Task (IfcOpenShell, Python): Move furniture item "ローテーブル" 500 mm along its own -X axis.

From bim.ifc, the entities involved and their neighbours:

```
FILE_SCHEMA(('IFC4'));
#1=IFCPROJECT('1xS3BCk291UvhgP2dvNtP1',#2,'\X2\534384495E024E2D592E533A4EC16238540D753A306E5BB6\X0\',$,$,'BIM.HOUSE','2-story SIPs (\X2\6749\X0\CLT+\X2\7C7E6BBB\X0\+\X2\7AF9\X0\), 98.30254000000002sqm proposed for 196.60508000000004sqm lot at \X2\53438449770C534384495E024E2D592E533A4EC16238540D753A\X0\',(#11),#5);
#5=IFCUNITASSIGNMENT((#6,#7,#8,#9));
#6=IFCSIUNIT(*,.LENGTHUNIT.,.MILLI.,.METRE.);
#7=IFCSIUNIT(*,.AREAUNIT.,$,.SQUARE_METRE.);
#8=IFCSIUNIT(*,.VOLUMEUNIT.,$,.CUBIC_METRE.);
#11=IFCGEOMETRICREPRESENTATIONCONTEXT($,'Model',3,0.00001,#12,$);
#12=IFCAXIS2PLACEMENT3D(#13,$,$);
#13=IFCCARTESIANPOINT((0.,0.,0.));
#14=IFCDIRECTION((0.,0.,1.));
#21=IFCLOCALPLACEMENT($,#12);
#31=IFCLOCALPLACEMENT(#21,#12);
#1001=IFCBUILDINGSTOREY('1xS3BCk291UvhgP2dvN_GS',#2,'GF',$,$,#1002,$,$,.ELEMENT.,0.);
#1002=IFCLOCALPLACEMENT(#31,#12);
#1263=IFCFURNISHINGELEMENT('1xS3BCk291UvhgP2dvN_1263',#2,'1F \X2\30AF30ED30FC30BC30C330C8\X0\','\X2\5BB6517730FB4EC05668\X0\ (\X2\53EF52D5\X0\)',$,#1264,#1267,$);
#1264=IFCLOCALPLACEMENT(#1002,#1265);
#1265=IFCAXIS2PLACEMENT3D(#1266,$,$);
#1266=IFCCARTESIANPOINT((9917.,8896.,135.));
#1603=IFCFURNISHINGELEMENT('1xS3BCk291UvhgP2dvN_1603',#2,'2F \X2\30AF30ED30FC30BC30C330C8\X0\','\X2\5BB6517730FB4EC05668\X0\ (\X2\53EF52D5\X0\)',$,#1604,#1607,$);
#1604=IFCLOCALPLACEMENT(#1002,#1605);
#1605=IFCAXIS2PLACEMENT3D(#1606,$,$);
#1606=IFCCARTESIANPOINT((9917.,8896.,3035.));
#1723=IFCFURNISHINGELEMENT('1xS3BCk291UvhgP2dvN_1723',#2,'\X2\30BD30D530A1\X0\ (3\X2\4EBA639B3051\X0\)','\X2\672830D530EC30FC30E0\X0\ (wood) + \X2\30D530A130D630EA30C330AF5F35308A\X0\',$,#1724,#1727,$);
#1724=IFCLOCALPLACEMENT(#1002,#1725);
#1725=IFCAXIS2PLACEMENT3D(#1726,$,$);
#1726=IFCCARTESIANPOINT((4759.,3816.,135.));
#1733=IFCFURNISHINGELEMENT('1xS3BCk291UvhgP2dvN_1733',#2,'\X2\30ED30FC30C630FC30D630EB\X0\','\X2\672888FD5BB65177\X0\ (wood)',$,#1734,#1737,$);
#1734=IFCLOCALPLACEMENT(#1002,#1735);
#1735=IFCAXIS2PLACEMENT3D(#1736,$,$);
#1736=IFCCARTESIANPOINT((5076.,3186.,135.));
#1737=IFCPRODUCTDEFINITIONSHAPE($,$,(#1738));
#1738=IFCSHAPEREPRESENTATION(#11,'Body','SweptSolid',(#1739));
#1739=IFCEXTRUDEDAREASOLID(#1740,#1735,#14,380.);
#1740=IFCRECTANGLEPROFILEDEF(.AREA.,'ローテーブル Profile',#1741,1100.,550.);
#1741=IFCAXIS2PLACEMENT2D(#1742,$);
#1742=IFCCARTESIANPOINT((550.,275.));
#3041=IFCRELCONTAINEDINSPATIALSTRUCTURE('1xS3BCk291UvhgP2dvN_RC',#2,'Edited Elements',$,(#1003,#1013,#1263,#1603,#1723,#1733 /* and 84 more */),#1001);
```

```python
import ifcopenshell
import ifcopenshell.api.geometry
import ifcopenshell.util.placement

model = ifcopenshell.open("bim.ifc")

item = model.by_id(1733)
matrix = ifcopenshell.util.placement.get_local_placement(item.ObjectPlacement)
matrix[:3, 3] -= matrix[:3, 0] * 500.0
ifcopenshell.api.geometry.edit_object_placement(model, product=item, matrix=matrix, is_si=False)

print(ifcopenshell.util.placement.get_local_placement(item.ObjectPlacement).round(3) + 0.0)

model.write("bim_v2.ifc")
```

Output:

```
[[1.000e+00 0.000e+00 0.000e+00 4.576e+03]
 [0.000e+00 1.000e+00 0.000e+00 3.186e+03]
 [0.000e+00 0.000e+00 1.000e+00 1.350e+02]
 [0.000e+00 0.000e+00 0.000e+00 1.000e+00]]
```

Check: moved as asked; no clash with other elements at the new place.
